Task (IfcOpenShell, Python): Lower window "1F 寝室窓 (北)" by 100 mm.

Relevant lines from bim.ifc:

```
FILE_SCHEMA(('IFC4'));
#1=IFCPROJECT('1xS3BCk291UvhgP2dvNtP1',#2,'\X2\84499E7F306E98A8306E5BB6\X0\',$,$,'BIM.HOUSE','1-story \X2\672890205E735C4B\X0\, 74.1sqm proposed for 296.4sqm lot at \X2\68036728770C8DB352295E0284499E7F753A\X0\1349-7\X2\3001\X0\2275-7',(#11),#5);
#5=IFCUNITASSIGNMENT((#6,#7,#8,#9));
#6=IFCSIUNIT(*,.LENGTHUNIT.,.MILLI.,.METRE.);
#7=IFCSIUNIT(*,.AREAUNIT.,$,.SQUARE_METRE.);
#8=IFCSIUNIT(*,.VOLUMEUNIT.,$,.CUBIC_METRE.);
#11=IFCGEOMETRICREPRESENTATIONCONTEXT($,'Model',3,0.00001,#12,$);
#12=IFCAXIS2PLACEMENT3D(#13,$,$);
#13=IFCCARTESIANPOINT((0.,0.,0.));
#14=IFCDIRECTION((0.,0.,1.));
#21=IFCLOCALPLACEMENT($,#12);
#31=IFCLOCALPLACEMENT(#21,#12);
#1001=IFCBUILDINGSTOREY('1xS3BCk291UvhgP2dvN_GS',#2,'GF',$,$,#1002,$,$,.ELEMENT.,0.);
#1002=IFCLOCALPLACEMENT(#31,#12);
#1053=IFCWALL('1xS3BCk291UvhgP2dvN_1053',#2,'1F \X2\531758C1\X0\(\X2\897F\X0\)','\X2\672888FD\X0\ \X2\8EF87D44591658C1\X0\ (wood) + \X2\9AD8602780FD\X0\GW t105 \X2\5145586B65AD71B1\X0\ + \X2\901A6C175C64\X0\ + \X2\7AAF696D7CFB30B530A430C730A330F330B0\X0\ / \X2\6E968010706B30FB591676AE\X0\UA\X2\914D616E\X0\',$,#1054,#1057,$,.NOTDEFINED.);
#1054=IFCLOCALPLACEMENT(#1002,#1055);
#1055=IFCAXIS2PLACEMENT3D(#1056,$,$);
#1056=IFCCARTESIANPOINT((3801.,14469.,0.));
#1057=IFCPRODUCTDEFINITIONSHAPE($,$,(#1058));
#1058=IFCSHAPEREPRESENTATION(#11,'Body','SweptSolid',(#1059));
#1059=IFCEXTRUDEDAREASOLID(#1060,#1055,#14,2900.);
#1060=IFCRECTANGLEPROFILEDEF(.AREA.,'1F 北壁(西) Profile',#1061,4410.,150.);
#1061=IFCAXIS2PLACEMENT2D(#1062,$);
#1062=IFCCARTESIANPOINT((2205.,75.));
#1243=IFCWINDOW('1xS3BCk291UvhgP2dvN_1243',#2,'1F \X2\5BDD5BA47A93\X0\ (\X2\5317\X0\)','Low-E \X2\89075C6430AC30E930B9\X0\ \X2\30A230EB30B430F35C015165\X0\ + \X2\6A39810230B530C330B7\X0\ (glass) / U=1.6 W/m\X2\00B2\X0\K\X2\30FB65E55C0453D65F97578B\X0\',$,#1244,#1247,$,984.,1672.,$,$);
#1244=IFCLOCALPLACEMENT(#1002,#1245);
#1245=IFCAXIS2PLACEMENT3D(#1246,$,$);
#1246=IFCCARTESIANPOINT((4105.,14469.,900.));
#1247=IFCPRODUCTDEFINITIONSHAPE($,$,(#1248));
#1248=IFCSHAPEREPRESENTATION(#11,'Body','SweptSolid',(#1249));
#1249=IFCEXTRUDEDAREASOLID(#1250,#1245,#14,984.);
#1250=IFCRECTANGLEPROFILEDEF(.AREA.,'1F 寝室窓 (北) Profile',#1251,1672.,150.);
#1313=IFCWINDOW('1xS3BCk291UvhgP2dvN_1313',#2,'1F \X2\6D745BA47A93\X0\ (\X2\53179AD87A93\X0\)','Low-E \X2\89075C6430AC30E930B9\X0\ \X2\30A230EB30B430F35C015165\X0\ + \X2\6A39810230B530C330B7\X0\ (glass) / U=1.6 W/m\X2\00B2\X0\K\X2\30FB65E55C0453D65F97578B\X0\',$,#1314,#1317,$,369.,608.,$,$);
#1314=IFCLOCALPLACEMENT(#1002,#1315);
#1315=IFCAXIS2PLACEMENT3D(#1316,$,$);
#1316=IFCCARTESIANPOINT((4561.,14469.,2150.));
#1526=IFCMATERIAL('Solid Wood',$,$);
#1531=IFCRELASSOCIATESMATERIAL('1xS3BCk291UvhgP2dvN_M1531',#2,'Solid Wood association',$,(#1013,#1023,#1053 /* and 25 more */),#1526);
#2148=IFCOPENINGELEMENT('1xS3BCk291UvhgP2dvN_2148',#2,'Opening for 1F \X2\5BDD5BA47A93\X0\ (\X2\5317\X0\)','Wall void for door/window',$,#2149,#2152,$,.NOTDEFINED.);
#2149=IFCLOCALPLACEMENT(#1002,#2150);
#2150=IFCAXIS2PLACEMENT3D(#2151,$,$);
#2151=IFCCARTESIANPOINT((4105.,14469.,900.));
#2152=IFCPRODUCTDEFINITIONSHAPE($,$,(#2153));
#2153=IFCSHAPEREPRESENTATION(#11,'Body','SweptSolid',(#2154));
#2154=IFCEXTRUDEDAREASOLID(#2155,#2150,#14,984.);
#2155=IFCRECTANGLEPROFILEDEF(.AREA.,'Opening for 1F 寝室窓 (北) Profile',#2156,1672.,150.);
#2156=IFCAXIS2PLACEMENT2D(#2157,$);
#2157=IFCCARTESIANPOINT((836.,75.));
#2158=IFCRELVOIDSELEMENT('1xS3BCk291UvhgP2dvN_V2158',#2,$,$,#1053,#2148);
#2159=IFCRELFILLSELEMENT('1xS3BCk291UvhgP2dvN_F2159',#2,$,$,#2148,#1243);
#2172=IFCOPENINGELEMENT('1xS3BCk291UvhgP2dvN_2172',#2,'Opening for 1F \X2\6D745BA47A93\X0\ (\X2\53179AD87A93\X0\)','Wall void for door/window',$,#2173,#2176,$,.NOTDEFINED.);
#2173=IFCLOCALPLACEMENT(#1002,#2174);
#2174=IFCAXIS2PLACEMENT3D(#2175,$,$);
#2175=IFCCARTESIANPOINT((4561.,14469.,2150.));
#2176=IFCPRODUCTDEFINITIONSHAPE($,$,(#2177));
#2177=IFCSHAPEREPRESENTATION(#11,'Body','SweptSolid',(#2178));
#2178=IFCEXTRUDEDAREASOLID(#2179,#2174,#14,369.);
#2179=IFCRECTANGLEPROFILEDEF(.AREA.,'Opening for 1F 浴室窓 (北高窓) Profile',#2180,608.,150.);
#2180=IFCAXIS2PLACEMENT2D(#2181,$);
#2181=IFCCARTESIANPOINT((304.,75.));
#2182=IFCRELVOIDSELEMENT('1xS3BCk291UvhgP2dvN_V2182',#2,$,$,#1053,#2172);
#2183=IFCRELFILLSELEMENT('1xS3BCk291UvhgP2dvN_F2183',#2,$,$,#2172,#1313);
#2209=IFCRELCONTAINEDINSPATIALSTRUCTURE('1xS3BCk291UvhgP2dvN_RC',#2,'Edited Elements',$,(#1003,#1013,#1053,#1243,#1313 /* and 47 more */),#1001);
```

```python
import numpy as np
import ifcopenshell
import ifcopenshell.api.geometry
import ifcopenshell.util.placement
import ifcopenshell.util.unit

model = ifcopenshell.open("bim.ifc")
unit_scale = ifcopenshell.util.unit.calculate_unit_scale(model)

window = model.by_id(1243)
opening = window.FillsVoids[0].RelatingOpeningElement
dz = -100.0

shift = np.array([0.0, 0.0, dz])
# The window is not placed relative to its opening, so move both.
for product in (opening, window):
    matrix = ifcopenshell.util.placement.get_local_placement(product.ObjectPlacement)
    matrix[:3, 3] += shift
    ifcopenshell.api.geometry.edit_object_placement(model, product=product, matrix=matrix, is_si=False)

print(f"moved by {dz * unit_scale:+.3f} m")

model.write("bim_v2.ifc")
```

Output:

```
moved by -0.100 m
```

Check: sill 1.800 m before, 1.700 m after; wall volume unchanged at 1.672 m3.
